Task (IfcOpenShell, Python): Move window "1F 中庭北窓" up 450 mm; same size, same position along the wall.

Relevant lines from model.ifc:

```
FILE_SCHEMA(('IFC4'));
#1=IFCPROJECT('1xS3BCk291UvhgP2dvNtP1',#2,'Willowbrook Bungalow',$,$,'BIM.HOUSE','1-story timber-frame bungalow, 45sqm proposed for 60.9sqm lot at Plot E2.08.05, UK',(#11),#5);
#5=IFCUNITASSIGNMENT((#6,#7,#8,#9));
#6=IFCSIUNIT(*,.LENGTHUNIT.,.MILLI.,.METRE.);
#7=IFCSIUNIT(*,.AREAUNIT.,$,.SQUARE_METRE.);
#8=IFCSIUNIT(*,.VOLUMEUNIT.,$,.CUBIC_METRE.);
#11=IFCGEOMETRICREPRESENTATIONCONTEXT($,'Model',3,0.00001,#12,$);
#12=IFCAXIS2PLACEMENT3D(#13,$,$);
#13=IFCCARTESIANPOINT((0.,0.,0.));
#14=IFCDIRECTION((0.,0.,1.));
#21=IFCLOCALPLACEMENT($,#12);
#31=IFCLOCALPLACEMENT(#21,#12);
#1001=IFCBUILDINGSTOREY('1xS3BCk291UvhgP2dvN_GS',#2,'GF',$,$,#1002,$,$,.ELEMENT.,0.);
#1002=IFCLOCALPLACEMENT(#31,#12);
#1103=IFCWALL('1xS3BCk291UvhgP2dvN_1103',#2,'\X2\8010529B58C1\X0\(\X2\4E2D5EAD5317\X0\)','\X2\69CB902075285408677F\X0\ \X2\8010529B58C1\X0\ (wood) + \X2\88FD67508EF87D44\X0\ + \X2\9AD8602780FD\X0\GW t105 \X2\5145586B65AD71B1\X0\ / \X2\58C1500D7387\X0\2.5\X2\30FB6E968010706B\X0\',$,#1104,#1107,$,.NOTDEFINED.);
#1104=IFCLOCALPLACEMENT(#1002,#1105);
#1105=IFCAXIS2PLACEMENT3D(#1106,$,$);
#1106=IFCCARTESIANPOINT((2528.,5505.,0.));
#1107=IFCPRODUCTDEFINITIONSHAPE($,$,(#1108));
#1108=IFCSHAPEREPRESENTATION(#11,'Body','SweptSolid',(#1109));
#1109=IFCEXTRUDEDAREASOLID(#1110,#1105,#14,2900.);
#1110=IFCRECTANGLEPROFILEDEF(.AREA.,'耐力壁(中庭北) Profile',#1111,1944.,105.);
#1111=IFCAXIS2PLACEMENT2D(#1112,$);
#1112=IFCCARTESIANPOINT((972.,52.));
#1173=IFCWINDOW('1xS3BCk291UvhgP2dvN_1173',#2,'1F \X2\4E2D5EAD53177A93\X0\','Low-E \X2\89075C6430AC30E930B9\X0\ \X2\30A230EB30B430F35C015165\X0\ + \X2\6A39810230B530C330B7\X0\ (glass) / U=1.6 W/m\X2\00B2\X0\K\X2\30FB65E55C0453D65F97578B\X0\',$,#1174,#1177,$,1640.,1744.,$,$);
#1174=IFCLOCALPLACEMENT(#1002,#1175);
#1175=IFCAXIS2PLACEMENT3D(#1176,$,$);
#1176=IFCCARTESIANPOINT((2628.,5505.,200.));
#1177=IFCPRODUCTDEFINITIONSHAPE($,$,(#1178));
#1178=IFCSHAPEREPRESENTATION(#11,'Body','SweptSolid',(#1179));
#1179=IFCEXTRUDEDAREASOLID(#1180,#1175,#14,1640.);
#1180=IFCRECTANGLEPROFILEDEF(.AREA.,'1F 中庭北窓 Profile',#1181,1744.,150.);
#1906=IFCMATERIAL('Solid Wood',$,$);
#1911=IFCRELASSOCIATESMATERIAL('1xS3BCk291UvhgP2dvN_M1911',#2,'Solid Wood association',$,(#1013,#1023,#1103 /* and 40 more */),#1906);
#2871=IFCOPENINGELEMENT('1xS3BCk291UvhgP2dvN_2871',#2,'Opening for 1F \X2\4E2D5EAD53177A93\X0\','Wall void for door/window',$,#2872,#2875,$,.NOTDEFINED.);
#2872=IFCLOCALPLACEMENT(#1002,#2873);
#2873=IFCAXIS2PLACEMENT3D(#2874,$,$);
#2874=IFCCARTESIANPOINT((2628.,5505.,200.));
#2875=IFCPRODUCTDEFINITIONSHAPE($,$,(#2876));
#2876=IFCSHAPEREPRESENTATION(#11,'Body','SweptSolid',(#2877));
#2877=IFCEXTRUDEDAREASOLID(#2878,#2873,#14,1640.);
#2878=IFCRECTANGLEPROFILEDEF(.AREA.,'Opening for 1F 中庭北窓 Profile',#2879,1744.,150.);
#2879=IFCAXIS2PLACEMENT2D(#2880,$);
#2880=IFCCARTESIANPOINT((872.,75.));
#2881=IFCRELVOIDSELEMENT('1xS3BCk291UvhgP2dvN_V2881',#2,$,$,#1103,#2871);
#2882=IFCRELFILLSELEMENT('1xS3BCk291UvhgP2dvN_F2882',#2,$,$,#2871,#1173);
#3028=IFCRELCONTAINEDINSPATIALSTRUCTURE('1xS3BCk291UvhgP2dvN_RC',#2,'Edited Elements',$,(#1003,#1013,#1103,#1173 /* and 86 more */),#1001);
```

```python
import numpy as np
import ifcopenshell
import ifcopenshell.api.geometry
import ifcopenshell.util.placement
import ifcopenshell.util.unit

model = ifcopenshell.open("model.ifc")
unit_scale = ifcopenshell.util.unit.calculate_unit_scale(model)

window = model.by_id(1173)
opening = window.FillsVoids[0].RelatingOpeningElement
dz = 0.45 / unit_scale

shift = np.array([0.0, 0.0, dz])
# The window is not placed relative to its opening, so move both.
for product in (opening, window):
    matrix = ifcopenshell.util.placement.get_local_placement(product.ObjectPlacement)
    matrix[:3, 3] += shift
    ifcopenshell.api.geometry.edit_object_placement(model, product=product, matrix=matrix, is_si=False)

print(f"moved by {dz * unit_scale:+.3f} m")

model.write("model_rev.ifc")
```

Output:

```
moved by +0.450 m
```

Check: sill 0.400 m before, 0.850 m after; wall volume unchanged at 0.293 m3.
